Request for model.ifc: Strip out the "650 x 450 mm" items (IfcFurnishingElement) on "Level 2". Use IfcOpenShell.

First a look at what the model holds.

```python
import ifcopenshell
import ifcopenshell.util.element

model = ifcopenshell.open("model.ifc")
print(model.schema)
storey = next(s for s in model.by_type("IfcBuildingStorey") if s.Name == "Level 2")
furniture = [e for e in ifcopenshell.util.element.get_decomposition(storey) if e.is_a("IfcFurnishingElement")]
seen = {}
for e in furniture:
    element_type = ifcopenshell.util.element.get_type(e)
    name = element_type.Name if element_type not in (None, e) else None
    seen[name] = seen.get(name, 0) + 1
for name, count in sorted(seen.items(), key=str):
    print(count, "x", name)
```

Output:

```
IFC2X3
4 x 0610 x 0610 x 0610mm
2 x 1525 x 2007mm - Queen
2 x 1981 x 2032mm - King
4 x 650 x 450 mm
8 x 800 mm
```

```python
import ifcopenshell
import ifcopenshell.api.root
import ifcopenshell.util.element

model = ifcopenshell.open("model.ifc")

storey = next(s for s in model.by_type("IfcBuildingStorey") if s.Name == "Level 2")
furniture = [e for e in ifcopenshell.util.element.get_decomposition(storey) if e.is_a("IfcFurnishingElement")]
targets = [e for e in furniture if (t := ifcopenshell.util.element.get_type(e)) not in (None, e) and t.Name == "650 x 450 mm"]

for e in targets:
    ifcopenshell.api.root.remove_product(model, product=e)
print(len(targets), "removed")

model.write("model-out.ifc")
```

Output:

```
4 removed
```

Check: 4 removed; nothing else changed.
